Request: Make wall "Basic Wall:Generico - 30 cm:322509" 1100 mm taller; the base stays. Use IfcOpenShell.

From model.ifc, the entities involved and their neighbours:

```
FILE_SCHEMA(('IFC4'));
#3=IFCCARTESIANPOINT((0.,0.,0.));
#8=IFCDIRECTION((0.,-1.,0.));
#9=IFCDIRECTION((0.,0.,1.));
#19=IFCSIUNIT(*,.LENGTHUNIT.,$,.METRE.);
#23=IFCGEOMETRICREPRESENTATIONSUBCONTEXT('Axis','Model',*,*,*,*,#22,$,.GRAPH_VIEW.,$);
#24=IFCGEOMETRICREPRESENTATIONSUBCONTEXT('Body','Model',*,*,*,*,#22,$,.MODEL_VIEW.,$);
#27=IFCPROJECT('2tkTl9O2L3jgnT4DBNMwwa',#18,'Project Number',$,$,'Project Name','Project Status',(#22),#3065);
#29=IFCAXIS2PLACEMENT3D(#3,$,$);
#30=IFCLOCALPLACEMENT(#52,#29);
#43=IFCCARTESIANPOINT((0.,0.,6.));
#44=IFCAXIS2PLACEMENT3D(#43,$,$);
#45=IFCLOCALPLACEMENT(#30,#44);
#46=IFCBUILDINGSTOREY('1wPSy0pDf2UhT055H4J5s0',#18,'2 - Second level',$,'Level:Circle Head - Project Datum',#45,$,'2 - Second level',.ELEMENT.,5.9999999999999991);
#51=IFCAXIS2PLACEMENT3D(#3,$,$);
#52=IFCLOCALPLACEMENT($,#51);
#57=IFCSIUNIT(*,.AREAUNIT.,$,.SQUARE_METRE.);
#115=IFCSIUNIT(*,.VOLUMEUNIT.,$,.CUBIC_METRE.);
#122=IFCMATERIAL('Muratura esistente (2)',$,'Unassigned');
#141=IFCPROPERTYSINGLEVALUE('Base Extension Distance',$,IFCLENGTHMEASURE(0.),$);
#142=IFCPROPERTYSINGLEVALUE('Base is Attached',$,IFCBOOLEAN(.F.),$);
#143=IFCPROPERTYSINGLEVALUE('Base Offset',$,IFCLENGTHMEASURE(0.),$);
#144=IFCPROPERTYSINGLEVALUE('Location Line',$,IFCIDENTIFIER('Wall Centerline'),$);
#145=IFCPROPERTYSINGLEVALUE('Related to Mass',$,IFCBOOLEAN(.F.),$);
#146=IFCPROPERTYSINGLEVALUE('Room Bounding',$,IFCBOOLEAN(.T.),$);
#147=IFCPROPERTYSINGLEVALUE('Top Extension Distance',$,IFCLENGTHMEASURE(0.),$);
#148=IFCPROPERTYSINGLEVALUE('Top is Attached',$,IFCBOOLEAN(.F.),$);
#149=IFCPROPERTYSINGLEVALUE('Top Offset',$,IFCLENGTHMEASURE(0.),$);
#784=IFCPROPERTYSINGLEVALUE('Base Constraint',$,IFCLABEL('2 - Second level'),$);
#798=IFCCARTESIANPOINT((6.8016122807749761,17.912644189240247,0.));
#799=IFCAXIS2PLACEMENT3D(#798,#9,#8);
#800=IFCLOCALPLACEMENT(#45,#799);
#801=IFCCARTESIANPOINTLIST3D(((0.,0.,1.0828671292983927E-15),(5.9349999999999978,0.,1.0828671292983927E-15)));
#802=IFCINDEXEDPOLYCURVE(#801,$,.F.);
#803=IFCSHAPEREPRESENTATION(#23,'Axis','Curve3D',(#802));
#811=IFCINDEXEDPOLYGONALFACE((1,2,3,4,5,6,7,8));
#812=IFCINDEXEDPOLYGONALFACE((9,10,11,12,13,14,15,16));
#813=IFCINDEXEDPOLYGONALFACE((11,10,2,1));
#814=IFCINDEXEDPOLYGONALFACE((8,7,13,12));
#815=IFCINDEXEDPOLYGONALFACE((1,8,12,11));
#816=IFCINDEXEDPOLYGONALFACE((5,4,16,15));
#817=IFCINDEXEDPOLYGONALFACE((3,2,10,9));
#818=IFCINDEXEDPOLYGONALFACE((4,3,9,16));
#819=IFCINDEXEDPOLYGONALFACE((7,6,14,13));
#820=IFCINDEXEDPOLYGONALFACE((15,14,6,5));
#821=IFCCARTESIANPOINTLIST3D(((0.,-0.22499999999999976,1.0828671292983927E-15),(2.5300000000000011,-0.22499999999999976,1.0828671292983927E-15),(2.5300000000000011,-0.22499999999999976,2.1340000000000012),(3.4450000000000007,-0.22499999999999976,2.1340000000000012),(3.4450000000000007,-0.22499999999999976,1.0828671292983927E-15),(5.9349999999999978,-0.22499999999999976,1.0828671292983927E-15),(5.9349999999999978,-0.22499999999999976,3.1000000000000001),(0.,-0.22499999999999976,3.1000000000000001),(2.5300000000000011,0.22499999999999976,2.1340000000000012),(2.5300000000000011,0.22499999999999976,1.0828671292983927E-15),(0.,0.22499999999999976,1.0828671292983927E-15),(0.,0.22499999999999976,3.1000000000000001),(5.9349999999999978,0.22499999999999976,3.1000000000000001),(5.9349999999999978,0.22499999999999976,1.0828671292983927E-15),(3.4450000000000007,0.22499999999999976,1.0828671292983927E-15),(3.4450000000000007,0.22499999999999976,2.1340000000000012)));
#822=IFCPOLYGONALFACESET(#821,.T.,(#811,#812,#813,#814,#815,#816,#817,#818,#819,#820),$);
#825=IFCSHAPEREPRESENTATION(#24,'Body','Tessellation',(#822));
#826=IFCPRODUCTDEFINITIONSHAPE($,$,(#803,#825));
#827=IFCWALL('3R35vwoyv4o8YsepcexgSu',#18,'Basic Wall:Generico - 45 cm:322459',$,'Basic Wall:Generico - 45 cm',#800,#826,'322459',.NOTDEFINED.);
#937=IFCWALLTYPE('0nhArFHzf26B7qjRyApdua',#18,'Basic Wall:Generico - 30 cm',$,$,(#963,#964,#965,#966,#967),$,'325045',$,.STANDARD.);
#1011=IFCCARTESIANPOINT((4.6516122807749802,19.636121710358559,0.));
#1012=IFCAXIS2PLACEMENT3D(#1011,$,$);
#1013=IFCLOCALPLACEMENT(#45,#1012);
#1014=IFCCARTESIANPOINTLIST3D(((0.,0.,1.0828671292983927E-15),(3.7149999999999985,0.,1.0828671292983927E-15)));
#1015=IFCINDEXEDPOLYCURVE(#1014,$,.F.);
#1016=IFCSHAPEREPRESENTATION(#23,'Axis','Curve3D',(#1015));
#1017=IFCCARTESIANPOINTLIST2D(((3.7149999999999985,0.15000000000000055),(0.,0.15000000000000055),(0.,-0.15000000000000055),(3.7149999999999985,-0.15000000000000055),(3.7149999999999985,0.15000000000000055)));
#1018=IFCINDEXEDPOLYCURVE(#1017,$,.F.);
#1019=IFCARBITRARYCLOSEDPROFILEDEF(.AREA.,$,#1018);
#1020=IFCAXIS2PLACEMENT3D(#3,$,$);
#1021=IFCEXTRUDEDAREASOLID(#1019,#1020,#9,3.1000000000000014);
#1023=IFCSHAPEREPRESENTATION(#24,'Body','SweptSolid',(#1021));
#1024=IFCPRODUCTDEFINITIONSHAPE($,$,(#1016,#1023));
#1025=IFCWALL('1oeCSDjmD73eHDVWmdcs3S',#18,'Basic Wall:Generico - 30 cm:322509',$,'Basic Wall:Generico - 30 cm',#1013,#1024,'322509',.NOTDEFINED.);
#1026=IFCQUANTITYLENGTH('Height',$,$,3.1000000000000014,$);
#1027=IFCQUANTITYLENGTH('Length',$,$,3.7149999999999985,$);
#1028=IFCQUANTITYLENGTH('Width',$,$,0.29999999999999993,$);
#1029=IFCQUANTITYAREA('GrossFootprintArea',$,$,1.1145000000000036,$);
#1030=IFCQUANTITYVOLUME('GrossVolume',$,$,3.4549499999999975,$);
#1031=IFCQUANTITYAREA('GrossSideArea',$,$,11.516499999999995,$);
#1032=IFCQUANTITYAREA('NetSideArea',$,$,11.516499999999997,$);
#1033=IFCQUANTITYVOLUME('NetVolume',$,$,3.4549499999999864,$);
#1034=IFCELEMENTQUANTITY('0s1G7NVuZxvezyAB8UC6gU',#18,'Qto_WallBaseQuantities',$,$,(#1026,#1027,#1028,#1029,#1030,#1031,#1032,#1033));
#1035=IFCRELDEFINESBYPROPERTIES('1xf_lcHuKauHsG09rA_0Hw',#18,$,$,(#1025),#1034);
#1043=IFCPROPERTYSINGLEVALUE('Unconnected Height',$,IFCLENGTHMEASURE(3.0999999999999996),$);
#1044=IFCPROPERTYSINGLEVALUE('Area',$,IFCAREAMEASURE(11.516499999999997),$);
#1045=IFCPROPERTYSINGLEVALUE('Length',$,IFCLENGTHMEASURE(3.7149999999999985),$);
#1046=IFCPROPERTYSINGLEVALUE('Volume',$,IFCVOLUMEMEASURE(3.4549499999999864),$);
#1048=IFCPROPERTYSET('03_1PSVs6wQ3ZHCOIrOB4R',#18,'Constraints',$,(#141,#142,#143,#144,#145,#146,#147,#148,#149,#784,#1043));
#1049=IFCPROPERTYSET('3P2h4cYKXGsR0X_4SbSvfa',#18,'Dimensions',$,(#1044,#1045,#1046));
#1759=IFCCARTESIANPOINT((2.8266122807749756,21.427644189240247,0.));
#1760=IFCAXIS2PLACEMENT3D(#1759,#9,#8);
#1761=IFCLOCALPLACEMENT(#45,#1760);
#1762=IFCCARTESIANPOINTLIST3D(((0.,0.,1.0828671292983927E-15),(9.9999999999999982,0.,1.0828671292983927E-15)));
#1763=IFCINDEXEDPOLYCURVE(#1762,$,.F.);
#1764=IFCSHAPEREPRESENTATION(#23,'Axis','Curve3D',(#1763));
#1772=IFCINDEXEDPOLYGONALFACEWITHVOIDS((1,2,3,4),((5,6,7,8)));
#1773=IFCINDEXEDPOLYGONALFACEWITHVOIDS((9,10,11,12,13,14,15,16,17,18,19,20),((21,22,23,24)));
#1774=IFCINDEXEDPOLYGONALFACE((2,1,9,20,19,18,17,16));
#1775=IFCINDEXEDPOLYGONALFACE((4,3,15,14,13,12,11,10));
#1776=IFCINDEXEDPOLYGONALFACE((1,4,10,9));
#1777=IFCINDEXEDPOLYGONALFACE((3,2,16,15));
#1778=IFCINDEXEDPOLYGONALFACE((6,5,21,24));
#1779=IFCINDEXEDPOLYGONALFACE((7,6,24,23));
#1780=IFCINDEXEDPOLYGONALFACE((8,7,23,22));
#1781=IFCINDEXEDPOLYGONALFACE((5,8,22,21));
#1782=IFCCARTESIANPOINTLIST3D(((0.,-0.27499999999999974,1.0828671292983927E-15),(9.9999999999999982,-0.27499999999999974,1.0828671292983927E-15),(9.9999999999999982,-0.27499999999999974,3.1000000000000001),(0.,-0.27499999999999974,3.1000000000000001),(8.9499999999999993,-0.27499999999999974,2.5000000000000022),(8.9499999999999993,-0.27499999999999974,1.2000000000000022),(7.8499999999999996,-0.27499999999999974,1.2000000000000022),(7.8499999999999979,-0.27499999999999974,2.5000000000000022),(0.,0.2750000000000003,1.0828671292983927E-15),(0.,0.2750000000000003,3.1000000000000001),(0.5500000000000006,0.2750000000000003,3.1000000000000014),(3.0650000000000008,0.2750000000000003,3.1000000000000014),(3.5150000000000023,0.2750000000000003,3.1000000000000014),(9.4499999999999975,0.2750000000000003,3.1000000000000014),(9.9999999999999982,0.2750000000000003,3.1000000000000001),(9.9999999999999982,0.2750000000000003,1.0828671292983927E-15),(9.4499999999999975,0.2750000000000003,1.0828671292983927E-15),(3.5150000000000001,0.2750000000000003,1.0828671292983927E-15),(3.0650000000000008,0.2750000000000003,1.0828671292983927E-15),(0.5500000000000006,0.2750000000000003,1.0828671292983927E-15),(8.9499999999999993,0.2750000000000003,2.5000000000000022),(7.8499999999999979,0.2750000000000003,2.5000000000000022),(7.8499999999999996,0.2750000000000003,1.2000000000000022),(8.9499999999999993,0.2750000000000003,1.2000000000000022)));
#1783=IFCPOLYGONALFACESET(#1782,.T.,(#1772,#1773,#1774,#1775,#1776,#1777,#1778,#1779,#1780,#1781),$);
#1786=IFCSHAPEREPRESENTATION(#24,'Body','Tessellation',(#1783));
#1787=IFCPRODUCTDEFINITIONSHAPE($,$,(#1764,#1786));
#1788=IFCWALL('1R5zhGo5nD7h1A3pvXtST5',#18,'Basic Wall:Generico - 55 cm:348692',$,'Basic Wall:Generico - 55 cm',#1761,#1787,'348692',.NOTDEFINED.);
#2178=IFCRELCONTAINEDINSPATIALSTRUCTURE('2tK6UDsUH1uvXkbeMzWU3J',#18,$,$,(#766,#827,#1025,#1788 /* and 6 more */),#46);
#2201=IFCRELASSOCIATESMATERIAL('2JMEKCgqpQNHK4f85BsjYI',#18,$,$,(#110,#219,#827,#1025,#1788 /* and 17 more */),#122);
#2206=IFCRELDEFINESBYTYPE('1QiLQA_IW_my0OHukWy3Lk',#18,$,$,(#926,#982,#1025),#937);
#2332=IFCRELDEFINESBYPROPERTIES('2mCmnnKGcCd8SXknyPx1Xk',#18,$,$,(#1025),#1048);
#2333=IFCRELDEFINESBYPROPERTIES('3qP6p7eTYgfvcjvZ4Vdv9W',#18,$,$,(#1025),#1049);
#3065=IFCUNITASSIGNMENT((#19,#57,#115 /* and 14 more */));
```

```python
import ifcopenshell
import ifcopenshell.api.pset
import ifcopenshell.geom
import ifcopenshell.util.element
import ifcopenshell.util.representation
import ifcopenshell.util.shape
import ifcopenshell.util.unit

model = ifcopenshell.open("model.ifc")
unit_scale = ifcopenshell.util.unit.calculate_unit_scale(model)
area_scale = ifcopenshell.util.unit.calculate_unit_scale(model, "AREAUNIT")
volume_scale = ifcopenshell.util.unit.calculate_unit_scale(model, "VOLUMEUNIT")
settings = ifcopenshell.geom.settings()


def volume(element):
    """Net volume in cubic metres, openings subtracted."""
    shape = ifcopenshell.geom.create_shape(settings, element)
    return ifcopenshell.util.shape.get_volume(shape.geometry)


wall = model.by_guid("1oeCSDjmD73eHDVWmdcs3S")
before = volume(wall)

body = ifcopenshell.util.representation.get_representation(wall, "Model", "Body")
solid = body.Items[0]
old_height = solid.Depth
solid.Depth += 1.1
after = volume(wall)
thickness = 0.3  # wall thickness in metres

# Update the stored height, areas and volumes.
qto = model.by_id(ifcopenshell.util.element.get_pset(wall, "Qto_WallBaseQuantities", should_inherit=False)["id"])
ifcopenshell.api.pset.edit_qto(model, qto=qto, properties={
    "Height": solid.Depth,
    "GrossVolume": ifcopenshell.util.element.get_pset(wall, "Qto_WallBaseQuantities", "GrossVolume") * solid.Depth / old_height,
    "GrossSideArea": ifcopenshell.util.element.get_pset(wall, "Qto_WallBaseQuantities", "GrossSideArea") * solid.Depth / old_height,
    "NetSideArea": after / thickness / area_scale,
    "NetVolume": after / volume_scale,
})
pset = model.by_id(ifcopenshell.util.element.get_pset(wall, "Constraints", should_inherit=False)["id"])
ifcopenshell.api.pset.edit_pset(model, pset=pset, properties={
    "Unconnected Height": model.create_entity("IfcLengthMeasure", solid.Depth),
})
pset = model.by_id(ifcopenshell.util.element.get_pset(wall, "Dimensions", should_inherit=False)["id"])
ifcopenshell.api.pset.edit_pset(model, pset=pset, properties={
    "Area": model.create_entity("IfcAreaMeasure", after / thickness / area_scale),
    "Volume": model.create_entity("IfcVolumeMeasure", after / volume_scale),
})

print(f"height {old_height:g} -> {solid.Depth:g}, volume {before:.3f} -> {after:.3f} m3")

model.write("model-out.ifc")
```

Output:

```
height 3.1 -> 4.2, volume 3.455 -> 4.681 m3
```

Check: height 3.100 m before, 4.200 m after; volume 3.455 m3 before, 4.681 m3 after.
